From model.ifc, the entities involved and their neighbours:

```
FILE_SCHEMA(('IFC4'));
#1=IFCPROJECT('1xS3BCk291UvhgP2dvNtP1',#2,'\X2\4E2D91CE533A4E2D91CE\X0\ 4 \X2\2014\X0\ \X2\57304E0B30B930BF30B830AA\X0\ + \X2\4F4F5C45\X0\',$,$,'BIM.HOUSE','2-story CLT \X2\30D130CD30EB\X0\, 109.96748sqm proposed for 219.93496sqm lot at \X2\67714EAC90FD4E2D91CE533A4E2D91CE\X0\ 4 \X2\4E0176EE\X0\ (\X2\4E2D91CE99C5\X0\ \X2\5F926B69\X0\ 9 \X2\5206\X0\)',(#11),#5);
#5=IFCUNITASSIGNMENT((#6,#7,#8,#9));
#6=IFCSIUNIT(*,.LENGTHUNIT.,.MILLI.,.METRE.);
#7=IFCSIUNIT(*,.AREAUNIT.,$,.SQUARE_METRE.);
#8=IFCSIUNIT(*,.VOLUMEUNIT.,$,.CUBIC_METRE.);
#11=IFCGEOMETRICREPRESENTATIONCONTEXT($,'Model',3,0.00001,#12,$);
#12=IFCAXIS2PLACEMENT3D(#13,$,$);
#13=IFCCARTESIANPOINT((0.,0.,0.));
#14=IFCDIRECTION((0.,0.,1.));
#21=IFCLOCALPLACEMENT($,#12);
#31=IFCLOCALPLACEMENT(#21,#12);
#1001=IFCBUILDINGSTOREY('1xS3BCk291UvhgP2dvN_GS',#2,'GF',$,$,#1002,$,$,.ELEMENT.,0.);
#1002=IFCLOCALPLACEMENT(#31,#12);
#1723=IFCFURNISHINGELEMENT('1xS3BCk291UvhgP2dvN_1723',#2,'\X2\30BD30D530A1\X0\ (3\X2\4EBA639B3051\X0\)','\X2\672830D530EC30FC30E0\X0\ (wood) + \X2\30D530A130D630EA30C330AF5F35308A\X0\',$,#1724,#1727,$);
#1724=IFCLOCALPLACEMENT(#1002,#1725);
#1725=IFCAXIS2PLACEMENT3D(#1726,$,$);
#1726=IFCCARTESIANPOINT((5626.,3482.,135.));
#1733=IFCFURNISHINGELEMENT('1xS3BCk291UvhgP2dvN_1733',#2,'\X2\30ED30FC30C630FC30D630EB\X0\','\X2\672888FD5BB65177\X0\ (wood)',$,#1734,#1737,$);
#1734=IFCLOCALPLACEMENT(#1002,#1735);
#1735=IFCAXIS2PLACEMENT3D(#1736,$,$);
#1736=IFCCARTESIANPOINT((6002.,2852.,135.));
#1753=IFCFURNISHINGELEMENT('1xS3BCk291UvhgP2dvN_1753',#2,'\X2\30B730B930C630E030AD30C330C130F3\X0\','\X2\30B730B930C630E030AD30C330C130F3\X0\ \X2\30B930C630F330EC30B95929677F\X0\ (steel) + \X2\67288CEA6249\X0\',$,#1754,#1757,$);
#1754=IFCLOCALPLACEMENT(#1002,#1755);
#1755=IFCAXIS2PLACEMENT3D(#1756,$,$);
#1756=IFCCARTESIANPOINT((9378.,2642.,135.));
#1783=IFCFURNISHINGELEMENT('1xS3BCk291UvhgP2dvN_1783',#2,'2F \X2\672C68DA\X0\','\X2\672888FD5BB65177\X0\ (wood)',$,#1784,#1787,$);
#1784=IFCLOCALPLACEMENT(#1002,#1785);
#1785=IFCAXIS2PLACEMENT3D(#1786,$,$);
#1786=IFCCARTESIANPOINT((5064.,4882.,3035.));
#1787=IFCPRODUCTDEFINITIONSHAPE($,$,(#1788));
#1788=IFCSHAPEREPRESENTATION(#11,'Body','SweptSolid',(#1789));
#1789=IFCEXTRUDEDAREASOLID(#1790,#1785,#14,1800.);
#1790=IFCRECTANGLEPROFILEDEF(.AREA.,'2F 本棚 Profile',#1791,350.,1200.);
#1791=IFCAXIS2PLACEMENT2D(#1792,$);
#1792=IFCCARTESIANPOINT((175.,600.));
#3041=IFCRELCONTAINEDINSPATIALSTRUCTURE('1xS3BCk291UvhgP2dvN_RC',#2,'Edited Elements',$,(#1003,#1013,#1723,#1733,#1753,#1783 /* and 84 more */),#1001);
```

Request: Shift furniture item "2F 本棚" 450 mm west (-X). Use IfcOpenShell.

```python
import ifcopenshell
import ifcopenshell.api.geometry
import ifcopenshell.util.placement
import ifcopenshell.util.unit

model = ifcopenshell.open("model.ifc")
unit_scale = ifcopenshell.util.unit.calculate_unit_scale(model)

item = model.by_guid("1xS3BCk291UvhgP2dvN_1783")
matrix = ifcopenshell.util.placement.get_local_placement(item.ObjectPlacement)
matrix[0, 3] -= 0.45 / unit_scale
ifcopenshell.api.geometry.edit_object_placement(model, product=item, matrix=matrix, is_si=False)

print(ifcopenshell.util.placement.get_local_placement(item.ObjectPlacement).round(3) + 0.0)

model.write("model_v2.ifc")
```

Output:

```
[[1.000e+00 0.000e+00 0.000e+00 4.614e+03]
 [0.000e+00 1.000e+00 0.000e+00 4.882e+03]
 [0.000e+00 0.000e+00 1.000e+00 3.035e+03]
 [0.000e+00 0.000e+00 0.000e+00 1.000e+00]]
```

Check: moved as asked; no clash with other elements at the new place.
